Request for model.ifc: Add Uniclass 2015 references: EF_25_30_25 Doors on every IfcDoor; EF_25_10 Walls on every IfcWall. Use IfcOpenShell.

First a look at what the model holds.

```python
import ifcopenshell

model = ifcopenshell.open("model.ifc")
print(model.schema)
print("classifications:", [c.Name for c in model.by_type("IfcClassification")])
for ifc_class in ("IfcDoor", "IfcRoof", "IfcStair", "IfcWall", "IfcWindow"):
    print(ifc_class, len(model.by_type(ifc_class)))
```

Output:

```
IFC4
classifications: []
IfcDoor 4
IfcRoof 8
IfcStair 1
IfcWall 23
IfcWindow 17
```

```python
import ifcopenshell
import ifcopenshell.api.classification

model = ifcopenshell.open("model.ifc")

system = ifcopenshell.api.classification.add_classification(model, classification="Uniclass 2015")

codes = {
    "IfcDoor": ("EF_25_30_25", "Doors"),
    "IfcWall": ("EF_25_10", "Walls"),
}
for ifc_class, (code, name) in codes.items():
    products = model.by_type(ifc_class)
    ifcopenshell.api.classification.add_reference(
        model, products=products, classification=system, identification=code, name=name
    )
    print(code, len(products))

model.write("model_v2.ifc")
```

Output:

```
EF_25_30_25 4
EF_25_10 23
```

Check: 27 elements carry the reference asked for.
